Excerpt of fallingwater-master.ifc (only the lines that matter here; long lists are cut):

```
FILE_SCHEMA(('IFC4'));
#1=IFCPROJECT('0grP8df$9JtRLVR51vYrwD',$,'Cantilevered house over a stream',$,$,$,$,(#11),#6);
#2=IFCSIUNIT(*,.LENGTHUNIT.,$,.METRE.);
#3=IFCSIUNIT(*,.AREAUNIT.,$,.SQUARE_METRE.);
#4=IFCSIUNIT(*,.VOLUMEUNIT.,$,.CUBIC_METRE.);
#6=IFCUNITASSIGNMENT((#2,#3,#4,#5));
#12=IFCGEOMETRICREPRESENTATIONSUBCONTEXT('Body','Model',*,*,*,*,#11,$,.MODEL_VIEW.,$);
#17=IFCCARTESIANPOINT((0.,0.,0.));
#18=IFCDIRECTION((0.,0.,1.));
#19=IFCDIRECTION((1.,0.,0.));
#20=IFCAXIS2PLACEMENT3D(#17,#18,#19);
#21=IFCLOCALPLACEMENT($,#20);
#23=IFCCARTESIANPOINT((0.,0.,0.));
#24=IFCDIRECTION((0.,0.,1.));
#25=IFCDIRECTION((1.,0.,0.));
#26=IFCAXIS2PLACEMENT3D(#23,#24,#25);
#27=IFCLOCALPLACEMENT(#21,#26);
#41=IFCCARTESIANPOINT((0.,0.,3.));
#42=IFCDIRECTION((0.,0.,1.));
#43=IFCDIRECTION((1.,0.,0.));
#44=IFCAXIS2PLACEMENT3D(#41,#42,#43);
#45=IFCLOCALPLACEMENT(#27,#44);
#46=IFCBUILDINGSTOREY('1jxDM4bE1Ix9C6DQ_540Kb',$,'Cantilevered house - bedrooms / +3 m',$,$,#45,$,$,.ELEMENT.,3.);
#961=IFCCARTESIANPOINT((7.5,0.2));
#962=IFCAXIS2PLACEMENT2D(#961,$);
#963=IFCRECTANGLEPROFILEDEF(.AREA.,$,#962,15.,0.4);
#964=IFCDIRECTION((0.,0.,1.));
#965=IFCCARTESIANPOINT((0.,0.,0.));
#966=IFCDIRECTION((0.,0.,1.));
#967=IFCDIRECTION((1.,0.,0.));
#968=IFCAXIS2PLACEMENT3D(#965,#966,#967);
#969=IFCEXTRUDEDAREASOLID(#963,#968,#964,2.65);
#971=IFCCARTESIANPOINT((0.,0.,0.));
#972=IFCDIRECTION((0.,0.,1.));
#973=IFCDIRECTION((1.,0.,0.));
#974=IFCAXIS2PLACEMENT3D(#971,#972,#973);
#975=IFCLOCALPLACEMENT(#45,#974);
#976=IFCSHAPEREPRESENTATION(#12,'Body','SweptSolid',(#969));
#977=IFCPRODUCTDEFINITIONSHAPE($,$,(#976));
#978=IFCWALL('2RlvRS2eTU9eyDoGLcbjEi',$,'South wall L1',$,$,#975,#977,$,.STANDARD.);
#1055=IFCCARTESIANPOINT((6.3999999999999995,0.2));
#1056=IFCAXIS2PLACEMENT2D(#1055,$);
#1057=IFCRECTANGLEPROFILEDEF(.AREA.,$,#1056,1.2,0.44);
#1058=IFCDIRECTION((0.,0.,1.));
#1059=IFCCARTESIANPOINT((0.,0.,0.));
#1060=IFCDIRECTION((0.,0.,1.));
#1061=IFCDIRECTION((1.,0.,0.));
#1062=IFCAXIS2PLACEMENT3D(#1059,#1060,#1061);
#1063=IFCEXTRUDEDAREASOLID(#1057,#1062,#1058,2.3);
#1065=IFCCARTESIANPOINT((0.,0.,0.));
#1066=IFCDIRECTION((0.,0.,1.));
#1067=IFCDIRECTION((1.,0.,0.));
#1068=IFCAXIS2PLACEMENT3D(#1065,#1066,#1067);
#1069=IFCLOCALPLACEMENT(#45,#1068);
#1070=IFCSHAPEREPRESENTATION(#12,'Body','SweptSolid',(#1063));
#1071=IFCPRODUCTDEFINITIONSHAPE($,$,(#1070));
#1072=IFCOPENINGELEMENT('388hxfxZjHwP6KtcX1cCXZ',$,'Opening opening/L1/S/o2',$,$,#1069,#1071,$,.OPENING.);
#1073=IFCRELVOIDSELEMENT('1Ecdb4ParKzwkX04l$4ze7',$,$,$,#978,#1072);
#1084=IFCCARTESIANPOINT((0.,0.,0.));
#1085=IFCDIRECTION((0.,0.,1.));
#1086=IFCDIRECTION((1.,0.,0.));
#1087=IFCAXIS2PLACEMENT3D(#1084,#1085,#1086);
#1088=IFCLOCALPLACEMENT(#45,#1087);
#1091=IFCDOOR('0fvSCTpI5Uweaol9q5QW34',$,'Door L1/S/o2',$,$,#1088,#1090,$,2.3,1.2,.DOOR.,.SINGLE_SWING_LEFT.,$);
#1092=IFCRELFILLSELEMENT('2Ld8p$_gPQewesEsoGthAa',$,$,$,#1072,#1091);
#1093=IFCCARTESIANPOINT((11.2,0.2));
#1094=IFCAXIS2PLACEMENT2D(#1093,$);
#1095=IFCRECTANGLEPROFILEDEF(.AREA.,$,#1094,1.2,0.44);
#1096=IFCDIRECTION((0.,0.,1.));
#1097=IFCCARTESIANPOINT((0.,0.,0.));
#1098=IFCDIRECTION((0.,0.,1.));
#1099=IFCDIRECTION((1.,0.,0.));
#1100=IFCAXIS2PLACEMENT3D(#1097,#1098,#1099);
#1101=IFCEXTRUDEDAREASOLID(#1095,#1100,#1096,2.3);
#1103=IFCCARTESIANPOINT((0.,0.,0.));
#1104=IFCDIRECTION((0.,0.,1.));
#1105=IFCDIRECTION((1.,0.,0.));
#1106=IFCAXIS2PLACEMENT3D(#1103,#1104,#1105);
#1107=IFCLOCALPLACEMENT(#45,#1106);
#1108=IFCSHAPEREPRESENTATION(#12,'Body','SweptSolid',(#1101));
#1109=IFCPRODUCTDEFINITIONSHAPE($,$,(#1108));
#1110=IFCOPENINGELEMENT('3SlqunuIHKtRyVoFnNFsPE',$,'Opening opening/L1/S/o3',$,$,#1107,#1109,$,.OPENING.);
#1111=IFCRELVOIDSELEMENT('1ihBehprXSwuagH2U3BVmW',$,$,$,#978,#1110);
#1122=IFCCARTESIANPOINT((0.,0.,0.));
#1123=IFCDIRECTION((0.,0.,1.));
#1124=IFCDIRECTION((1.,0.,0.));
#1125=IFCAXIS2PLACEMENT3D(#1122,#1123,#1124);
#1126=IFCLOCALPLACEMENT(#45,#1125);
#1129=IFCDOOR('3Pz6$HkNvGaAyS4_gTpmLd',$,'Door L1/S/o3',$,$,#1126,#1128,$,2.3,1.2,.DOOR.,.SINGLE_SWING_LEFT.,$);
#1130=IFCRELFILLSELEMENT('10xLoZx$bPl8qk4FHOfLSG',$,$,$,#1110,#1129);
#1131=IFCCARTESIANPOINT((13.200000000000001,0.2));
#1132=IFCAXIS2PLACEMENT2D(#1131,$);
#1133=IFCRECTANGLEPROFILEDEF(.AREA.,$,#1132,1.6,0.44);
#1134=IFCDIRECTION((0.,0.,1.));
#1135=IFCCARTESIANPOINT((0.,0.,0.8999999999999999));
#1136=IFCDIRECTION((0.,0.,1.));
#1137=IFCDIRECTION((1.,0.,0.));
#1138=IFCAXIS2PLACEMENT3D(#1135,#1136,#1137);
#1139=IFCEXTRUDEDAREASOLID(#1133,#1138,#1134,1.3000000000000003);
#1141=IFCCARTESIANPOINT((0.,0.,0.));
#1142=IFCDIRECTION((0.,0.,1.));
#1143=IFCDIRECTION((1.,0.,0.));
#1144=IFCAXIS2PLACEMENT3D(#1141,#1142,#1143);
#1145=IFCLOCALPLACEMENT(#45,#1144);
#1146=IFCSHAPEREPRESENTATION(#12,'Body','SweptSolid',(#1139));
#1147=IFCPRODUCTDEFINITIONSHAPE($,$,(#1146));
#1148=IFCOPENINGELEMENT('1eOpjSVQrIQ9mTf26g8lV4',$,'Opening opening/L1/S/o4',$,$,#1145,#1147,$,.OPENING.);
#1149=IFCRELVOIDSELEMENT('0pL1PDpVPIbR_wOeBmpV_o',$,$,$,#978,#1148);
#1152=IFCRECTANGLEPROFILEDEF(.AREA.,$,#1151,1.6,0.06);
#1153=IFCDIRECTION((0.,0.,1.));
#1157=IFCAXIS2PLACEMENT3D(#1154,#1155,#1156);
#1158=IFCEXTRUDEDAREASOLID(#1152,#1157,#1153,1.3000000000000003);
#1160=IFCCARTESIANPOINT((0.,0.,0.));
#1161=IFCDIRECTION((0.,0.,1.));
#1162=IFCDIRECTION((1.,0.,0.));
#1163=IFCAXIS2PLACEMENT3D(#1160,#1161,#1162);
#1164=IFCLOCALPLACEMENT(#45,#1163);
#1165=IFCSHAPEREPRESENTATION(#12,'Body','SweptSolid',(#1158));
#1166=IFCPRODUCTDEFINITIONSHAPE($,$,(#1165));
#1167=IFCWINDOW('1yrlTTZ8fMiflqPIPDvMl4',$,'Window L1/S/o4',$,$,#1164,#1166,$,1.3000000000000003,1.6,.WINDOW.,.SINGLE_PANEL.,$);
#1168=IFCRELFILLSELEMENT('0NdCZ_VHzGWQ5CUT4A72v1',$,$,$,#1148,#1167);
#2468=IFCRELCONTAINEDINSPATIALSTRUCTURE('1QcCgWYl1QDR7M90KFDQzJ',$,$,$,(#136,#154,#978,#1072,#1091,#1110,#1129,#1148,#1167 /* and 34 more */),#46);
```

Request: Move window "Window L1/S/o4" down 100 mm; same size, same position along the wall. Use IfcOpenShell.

```python
import numpy as np
import ifcopenshell
import ifcopenshell.api.geometry
import ifcopenshell.util.placement
import ifcopenshell.util.unit

model = ifcopenshell.open("fallingwater-master.ifc")
unit_scale = ifcopenshell.util.unit.calculate_unit_scale(model)

window = model.by_guid("1yrlTTZ8fMiflqPIPDvMl4")
opening = window.FillsVoids[0].RelatingOpeningElement
dz = -0.1

shift = np.array([0.0, 0.0, dz])
# The window is not placed relative to its opening, so move both.
for product in (opening, window):
    matrix = ifcopenshell.util.placement.get_local_placement(product.ObjectPlacement)
    matrix[:3, 3] += shift
    ifcopenshell.api.geometry.edit_object_placement(model, product=product, matrix=matrix, is_si=False)

print(f"moved by {dz * unit_scale:+.3f} m")

model.write("fallingwater-master_rev.ifc")
```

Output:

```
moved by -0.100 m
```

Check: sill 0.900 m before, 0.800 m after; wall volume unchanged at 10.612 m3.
